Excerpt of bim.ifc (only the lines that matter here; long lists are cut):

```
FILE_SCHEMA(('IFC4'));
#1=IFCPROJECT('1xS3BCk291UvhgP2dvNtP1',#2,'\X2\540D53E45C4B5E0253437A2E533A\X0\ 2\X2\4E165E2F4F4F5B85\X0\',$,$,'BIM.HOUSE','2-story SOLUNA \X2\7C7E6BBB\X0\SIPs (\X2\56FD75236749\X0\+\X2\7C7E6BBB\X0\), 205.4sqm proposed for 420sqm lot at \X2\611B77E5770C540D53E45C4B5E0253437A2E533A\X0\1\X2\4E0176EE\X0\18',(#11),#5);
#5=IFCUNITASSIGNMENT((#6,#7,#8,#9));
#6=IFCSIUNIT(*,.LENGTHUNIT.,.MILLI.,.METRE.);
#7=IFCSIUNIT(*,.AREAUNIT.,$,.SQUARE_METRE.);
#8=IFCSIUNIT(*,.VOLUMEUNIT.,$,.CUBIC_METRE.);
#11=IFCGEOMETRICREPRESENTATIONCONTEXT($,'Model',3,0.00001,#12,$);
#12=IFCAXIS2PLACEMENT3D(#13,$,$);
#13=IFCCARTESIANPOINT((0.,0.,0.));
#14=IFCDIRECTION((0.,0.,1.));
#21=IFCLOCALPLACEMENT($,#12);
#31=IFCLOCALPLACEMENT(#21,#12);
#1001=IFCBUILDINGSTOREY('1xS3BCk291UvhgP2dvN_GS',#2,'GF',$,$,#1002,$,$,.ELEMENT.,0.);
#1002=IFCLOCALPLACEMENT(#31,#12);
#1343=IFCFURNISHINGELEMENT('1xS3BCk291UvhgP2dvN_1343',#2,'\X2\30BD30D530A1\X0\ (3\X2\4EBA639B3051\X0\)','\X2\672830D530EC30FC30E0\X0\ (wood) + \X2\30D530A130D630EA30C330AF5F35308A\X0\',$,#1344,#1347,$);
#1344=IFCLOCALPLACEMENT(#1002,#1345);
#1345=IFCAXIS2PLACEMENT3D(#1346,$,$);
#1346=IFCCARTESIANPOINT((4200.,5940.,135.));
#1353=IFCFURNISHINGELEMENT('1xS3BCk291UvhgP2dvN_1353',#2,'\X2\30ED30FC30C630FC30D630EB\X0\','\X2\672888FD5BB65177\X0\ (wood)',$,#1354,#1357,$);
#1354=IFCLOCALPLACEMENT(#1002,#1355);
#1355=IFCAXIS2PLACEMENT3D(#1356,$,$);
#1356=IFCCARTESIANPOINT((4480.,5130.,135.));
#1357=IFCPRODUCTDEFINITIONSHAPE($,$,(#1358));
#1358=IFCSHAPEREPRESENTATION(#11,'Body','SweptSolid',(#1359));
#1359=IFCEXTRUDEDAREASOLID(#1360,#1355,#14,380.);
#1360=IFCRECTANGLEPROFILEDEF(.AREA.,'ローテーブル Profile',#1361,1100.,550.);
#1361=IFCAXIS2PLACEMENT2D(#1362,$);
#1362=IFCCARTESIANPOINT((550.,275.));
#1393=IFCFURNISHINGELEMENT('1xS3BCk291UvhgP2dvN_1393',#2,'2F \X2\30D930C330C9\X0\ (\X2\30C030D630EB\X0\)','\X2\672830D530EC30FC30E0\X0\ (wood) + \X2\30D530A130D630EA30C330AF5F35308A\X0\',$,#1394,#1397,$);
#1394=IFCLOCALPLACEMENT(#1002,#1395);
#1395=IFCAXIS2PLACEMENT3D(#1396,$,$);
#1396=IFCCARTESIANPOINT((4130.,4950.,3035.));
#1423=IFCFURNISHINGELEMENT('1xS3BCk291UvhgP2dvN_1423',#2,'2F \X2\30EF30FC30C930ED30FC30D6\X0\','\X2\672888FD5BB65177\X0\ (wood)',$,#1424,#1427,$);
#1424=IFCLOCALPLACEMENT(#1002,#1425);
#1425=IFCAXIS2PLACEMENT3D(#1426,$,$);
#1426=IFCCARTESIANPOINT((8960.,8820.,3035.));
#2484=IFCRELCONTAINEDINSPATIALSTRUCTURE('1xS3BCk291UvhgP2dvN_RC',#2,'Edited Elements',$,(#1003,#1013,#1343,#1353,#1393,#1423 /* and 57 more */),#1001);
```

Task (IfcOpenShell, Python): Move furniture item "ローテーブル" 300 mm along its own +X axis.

```python
import ifcopenshell
import ifcopenshell.api.geometry
import ifcopenshell.util.placement

model = ifcopenshell.open("bim.ifc")

item = model.by_guid("1xS3BCk291UvhgP2dvN_1353")
matrix = ifcopenshell.util.placement.get_local_placement(item.ObjectPlacement)
matrix[:3, 3] += matrix[:3, 0] * 300.0
ifcopenshell.api.geometry.edit_object_placement(model, product=item, matrix=matrix, is_si=False)

print(ifcopenshell.util.placement.get_local_placement(item.ObjectPlacement).round(3) + 0.0)

model.write("bim-out.ifc")
```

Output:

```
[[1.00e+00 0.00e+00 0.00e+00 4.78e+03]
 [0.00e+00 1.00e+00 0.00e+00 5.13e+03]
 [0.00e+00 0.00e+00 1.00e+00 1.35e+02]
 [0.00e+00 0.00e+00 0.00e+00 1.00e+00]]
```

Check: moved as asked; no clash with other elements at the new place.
